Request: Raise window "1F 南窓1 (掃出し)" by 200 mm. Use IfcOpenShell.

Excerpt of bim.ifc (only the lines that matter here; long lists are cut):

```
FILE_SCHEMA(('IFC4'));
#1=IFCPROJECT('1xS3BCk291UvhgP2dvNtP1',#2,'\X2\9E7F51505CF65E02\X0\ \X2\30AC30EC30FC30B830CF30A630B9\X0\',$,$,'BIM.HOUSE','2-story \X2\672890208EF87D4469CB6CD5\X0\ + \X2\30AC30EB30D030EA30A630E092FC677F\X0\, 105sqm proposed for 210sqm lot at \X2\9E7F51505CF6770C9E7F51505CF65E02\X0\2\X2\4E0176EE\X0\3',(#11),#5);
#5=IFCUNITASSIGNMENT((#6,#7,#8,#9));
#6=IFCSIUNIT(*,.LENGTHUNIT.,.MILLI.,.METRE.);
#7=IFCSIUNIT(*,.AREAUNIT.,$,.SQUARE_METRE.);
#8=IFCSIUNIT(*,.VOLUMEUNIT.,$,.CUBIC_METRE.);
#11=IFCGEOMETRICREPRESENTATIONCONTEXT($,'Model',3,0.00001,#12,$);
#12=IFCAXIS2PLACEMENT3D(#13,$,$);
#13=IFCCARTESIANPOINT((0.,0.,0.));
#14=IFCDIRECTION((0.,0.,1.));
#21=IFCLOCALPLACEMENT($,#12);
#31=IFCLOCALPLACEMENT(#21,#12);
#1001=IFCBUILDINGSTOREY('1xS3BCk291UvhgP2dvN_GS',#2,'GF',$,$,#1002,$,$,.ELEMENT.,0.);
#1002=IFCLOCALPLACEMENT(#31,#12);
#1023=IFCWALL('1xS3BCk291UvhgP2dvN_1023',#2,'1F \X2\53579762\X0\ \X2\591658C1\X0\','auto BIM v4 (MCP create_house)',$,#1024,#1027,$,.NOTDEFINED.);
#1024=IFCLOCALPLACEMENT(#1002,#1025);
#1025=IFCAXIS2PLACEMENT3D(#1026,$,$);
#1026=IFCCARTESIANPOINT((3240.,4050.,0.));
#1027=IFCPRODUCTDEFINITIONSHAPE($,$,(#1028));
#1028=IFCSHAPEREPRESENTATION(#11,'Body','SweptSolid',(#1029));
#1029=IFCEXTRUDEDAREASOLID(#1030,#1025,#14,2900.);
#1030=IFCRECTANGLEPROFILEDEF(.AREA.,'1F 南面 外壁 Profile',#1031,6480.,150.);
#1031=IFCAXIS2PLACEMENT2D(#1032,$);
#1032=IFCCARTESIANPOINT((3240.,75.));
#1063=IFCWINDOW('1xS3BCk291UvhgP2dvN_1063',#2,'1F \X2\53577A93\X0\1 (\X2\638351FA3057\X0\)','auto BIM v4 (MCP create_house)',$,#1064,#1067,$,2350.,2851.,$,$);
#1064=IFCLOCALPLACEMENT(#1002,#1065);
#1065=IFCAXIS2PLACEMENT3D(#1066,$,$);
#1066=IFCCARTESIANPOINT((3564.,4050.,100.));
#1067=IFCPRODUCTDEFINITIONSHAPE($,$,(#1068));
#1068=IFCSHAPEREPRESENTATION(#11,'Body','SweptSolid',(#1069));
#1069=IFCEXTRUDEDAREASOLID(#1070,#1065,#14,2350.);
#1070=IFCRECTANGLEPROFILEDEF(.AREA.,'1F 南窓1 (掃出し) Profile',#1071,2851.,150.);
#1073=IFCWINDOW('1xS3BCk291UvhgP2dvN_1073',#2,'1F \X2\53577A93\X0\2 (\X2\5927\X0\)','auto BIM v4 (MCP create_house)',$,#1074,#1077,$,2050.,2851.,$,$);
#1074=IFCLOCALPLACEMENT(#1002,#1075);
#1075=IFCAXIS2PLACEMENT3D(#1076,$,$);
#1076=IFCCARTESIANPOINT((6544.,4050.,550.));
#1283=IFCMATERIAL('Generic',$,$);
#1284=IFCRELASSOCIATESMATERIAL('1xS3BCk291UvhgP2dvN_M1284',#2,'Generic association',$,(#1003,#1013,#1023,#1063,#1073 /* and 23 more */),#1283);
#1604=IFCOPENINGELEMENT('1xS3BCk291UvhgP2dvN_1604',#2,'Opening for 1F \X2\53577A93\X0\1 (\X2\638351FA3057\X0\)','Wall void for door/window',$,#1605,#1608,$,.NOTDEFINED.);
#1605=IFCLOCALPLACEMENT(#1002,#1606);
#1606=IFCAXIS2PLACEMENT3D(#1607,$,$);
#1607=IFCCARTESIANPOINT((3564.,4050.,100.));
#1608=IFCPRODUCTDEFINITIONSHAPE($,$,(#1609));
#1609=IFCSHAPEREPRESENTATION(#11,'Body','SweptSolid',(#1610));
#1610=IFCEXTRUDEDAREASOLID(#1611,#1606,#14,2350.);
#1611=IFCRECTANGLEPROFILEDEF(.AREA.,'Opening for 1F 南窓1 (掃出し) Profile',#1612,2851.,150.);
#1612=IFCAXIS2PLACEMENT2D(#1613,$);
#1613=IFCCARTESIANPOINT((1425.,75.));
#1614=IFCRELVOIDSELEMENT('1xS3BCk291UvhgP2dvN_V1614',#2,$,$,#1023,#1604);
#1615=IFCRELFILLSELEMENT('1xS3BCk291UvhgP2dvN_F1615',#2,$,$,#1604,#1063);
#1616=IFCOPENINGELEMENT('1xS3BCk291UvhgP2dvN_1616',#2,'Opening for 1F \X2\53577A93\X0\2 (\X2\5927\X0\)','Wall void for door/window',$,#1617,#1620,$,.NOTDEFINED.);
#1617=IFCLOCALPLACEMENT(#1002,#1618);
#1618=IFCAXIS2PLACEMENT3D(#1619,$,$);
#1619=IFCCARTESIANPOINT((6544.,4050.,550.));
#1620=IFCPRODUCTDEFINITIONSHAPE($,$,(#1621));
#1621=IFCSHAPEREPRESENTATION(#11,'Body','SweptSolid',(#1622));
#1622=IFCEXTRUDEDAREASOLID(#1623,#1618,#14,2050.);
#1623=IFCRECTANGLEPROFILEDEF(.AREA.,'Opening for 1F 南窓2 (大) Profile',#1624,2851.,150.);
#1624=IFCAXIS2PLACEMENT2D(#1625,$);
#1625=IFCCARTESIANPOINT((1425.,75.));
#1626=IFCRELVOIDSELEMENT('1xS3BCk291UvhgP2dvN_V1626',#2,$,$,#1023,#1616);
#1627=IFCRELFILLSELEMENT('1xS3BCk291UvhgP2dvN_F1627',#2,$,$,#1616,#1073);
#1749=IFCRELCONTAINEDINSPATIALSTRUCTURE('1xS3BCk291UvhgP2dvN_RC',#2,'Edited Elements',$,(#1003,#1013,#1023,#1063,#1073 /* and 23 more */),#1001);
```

```python
import numpy as np
import ifcopenshell
import ifcopenshell.api.geometry
import ifcopenshell.util.placement
import ifcopenshell.util.unit

model = ifcopenshell.open("bim.ifc")
unit_scale = ifcopenshell.util.unit.calculate_unit_scale(model)

window = model.by_id(1063)
opening = window.FillsVoids[0].RelatingOpeningElement
dz = 200.0

shift = np.array([0.0, 0.0, dz])
# The window is not placed relative to its opening, so move both.
for product in (opening, window):
    matrix = ifcopenshell.util.placement.get_local_placement(product.ObjectPlacement)
    matrix[:3, 3] += shift
    ifcopenshell.api.geometry.edit_object_placement(model, product=product, matrix=matrix, is_si=False)

print(f"moved by {dz * unit_scale:+.3f} m")

model.write("bim_updated.ifc")
```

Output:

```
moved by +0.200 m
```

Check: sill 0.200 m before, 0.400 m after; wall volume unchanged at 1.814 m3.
